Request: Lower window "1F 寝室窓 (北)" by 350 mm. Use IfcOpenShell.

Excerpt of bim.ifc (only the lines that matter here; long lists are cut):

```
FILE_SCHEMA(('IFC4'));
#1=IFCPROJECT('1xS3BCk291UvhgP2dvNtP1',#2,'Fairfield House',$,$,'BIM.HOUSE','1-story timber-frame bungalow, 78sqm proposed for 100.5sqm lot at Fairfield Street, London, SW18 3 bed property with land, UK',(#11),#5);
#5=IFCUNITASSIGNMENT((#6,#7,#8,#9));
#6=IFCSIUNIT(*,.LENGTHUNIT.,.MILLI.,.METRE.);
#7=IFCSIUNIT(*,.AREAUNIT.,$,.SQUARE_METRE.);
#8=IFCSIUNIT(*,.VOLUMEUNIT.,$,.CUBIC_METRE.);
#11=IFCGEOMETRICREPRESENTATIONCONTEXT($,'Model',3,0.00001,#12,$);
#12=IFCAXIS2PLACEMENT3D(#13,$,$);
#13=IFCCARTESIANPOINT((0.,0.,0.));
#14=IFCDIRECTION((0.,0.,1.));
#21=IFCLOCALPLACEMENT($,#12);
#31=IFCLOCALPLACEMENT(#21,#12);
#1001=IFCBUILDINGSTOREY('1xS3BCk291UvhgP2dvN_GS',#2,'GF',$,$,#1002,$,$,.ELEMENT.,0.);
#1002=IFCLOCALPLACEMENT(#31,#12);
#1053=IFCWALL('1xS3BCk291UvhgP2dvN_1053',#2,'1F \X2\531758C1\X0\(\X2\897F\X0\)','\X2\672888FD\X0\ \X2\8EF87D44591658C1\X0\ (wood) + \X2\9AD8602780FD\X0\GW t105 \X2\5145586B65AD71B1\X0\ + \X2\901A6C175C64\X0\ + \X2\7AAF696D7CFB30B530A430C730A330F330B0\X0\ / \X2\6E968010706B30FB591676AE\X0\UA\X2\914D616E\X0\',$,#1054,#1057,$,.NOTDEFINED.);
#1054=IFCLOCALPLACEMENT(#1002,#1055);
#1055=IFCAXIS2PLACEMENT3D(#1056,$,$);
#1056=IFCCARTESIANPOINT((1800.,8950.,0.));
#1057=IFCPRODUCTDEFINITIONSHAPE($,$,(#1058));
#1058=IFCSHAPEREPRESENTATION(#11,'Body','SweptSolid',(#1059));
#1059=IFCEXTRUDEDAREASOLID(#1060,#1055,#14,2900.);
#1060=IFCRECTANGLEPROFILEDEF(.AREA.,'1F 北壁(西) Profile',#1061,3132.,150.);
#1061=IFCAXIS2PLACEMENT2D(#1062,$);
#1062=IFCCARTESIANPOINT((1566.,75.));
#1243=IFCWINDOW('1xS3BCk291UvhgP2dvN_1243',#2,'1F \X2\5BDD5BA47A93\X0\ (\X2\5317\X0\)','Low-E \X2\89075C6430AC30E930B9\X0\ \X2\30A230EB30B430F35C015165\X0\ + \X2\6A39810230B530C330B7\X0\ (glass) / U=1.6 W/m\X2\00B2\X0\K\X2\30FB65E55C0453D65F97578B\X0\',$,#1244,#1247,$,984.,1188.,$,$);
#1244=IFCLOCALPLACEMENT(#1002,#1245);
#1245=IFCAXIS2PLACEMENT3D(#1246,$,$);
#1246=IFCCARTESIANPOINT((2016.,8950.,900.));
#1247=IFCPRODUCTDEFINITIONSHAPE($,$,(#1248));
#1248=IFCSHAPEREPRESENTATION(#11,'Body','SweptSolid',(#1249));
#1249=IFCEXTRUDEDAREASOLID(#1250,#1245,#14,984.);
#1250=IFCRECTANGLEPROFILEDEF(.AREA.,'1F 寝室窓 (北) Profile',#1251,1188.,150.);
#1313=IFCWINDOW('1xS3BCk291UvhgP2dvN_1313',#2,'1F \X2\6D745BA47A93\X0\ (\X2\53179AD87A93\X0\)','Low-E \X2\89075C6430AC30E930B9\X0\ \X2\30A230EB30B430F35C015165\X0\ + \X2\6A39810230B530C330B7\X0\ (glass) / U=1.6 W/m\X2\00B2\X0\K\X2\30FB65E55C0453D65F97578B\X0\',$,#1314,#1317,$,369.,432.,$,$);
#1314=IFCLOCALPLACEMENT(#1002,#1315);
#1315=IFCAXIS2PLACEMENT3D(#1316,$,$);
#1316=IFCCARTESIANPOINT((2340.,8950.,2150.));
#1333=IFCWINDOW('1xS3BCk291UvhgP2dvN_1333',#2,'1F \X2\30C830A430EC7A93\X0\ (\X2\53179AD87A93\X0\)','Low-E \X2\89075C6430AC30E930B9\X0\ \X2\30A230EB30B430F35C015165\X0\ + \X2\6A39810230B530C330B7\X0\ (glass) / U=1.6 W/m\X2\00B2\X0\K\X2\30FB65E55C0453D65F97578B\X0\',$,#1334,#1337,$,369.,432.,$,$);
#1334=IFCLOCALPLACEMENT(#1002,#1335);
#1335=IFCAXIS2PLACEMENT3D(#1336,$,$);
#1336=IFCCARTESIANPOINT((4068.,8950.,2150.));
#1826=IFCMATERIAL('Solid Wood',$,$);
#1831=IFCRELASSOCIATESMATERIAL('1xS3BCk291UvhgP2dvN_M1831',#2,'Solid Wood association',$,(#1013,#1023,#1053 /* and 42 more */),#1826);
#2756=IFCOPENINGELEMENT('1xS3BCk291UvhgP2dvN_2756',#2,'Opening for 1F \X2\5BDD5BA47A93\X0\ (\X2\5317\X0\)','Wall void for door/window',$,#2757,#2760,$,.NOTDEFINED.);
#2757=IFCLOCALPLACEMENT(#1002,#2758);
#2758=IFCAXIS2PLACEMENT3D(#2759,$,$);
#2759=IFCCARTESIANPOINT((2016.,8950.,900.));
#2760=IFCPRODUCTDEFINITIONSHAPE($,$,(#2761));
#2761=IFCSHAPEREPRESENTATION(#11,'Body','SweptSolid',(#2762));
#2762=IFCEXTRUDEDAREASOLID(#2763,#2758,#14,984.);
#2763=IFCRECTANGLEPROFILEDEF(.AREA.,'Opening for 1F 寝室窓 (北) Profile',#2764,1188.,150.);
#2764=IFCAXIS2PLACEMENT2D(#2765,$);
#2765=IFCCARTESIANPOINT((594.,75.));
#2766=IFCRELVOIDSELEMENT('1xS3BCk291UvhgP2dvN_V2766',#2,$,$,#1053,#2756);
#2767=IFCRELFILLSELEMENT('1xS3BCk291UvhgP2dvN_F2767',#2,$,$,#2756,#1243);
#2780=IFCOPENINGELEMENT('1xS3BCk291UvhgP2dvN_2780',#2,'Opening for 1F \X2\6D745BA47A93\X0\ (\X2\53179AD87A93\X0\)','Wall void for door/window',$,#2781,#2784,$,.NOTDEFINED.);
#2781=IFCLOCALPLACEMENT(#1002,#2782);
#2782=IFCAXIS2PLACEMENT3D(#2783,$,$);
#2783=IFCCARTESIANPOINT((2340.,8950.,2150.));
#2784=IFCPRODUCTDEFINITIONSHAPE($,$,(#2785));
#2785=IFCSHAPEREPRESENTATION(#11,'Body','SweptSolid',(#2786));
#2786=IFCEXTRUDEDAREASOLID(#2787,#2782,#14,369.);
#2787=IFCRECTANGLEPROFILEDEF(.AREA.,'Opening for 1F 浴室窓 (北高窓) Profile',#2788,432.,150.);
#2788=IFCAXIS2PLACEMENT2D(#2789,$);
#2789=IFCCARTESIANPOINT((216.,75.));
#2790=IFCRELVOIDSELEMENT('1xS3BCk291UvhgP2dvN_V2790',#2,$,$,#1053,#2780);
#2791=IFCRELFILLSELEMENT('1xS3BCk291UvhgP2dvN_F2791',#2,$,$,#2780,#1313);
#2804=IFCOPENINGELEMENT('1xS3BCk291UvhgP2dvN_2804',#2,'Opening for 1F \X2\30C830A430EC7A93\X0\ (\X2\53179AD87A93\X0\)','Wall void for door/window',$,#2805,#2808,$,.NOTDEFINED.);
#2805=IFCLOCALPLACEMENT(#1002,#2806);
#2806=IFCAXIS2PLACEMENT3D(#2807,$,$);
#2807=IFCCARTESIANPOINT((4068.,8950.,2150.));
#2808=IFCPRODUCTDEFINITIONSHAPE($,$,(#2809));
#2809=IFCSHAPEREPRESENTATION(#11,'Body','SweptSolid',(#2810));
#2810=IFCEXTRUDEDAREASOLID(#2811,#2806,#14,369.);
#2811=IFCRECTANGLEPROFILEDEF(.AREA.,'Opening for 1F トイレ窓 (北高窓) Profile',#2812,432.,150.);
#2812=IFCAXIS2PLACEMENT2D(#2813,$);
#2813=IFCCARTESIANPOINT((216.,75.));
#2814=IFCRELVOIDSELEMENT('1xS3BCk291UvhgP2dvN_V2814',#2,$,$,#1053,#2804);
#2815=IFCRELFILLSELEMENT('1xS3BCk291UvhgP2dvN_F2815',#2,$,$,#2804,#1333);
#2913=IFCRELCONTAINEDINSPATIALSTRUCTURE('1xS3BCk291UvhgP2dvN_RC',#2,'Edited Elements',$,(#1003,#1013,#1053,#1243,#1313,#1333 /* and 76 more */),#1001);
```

```python
import numpy as np
import ifcopenshell
import ifcopenshell.api.geometry
import ifcopenshell.util.placement
import ifcopenshell.util.unit

model = ifcopenshell.open("bim.ifc")
unit_scale = ifcopenshell.util.unit.calculate_unit_scale(model)

window = model.by_guid("1xS3BCk291UvhgP2dvN_1243")
opening = window.FillsVoids[0].RelatingOpeningElement
dz = -0.35 / unit_scale

shift = np.array([0.0, 0.0, dz])
# The window is not placed relative to its opening, so move both.
for product in (opening, window):
    matrix = ifcopenshell.util.placement.get_local_placement(product.ObjectPlacement)
    matrix[:3, 3] += shift
    ifcopenshell.api.geometry.edit_object_placement(model, product=product, matrix=matrix, is_si=False)

print(f"moved by {dz * unit_scale:+.3f} m")

model.write("bim_edited.ifc")
```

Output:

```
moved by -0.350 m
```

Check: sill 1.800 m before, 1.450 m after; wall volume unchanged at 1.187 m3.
